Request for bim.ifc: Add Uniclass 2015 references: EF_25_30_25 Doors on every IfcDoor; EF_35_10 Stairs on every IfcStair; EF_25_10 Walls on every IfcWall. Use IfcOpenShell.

First a look at what the model holds.

```python
import ifcopenshell

model = ifcopenshell.open("bim.ifc")
print(model.schema)
print("classifications:", [c.Name for c in model.by_type("IfcClassification")])
for ifc_class in ("IfcDoor", "IfcRoof", "IfcStair", "IfcWall", "IfcWindow"):
    print(ifc_class, len(model.by_type(ifc_class)))
```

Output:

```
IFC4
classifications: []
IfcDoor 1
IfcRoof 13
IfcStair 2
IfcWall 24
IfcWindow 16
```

```python
import ifcopenshell
import ifcopenshell.api.classification

model = ifcopenshell.open("bim.ifc")

system = ifcopenshell.api.classification.add_classification(model, classification="Uniclass 2015")

codes = {
    "IfcDoor": ("EF_25_30_25", "Doors"),
    "IfcStair": ("EF_35_10", "Stairs"),
    "IfcWall": ("EF_25_10", "Walls"),
}
for ifc_class, (code, name) in codes.items():
    products = model.by_type(ifc_class)
    ifcopenshell.api.classification.add_reference(
        model, products=products, classification=system, identification=code, name=name
    )
    print(code, len(products))

model.write("bim_edited.ifc")
```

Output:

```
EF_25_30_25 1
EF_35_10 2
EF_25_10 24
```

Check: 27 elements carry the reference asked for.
